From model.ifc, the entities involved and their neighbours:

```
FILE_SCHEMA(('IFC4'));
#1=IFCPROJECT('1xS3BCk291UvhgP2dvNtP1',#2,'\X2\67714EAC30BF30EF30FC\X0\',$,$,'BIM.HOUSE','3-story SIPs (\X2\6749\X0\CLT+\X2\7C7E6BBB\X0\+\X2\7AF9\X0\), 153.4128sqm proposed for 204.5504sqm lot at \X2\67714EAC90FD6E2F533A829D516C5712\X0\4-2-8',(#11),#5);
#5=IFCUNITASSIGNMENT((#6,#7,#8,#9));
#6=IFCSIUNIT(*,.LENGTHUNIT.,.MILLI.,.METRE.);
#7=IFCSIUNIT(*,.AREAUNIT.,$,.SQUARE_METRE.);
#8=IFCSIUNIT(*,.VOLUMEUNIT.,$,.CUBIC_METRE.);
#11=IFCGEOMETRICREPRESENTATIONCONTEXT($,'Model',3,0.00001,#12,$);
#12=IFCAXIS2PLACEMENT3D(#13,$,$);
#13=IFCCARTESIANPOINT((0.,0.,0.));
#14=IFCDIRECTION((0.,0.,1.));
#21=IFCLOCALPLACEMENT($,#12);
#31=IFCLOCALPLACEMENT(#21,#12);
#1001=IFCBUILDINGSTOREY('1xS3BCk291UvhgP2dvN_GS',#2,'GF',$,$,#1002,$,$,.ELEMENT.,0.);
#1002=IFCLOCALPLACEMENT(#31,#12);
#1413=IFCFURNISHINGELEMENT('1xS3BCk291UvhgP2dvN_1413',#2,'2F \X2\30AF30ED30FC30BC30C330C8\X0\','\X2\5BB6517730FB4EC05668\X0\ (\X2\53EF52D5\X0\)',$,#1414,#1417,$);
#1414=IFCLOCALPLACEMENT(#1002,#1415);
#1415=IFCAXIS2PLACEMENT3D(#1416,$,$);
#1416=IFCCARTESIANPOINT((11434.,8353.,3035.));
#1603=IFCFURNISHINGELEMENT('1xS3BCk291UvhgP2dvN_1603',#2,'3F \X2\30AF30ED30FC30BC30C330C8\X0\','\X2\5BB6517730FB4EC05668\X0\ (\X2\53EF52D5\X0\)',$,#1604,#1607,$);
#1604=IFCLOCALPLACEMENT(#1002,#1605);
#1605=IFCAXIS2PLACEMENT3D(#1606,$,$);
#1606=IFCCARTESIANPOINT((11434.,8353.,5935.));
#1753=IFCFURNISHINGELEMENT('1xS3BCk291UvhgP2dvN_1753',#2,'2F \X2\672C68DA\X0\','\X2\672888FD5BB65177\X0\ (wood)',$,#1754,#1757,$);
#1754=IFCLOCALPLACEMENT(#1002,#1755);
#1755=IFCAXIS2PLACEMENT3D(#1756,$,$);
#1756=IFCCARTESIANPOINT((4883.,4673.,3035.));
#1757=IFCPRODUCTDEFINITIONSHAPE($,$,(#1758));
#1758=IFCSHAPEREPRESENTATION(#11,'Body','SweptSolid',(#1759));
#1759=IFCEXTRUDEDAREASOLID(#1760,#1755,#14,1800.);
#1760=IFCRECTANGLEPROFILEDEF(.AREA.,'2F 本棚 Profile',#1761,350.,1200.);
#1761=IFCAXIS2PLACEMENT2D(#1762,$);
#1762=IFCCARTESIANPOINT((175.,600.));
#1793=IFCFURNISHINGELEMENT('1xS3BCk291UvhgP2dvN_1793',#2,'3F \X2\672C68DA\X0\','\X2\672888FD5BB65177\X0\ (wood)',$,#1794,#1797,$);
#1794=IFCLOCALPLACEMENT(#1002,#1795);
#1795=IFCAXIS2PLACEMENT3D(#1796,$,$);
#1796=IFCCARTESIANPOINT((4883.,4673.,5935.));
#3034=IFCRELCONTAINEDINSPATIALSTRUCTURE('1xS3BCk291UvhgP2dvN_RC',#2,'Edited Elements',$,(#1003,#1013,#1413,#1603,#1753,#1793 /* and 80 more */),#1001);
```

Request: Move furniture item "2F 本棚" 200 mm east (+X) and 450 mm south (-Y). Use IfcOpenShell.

```python
import ifcopenshell
import ifcopenshell.api.geometry
import ifcopenshell.util.placement
import ifcopenshell.util.unit

model = ifcopenshell.open("model.ifc")
unit_scale = ifcopenshell.util.unit.calculate_unit_scale(model)

item = model.by_guid("1xS3BCk291UvhgP2dvN_1753")
matrix = ifcopenshell.util.placement.get_local_placement(item.ObjectPlacement)
matrix[0, 3] += 0.2 / unit_scale
matrix[1, 3] -= 0.45 / unit_scale
ifcopenshell.api.geometry.edit_object_placement(model, product=item, matrix=matrix, is_si=False)

print(ifcopenshell.util.placement.get_local_placement(item.ObjectPlacement).round(3) + 0.0)

model.write("model_v2.ifc")
```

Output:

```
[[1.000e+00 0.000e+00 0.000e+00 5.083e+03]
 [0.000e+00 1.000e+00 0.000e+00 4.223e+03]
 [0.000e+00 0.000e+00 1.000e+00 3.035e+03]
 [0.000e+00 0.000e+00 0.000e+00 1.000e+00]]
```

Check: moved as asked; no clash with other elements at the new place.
